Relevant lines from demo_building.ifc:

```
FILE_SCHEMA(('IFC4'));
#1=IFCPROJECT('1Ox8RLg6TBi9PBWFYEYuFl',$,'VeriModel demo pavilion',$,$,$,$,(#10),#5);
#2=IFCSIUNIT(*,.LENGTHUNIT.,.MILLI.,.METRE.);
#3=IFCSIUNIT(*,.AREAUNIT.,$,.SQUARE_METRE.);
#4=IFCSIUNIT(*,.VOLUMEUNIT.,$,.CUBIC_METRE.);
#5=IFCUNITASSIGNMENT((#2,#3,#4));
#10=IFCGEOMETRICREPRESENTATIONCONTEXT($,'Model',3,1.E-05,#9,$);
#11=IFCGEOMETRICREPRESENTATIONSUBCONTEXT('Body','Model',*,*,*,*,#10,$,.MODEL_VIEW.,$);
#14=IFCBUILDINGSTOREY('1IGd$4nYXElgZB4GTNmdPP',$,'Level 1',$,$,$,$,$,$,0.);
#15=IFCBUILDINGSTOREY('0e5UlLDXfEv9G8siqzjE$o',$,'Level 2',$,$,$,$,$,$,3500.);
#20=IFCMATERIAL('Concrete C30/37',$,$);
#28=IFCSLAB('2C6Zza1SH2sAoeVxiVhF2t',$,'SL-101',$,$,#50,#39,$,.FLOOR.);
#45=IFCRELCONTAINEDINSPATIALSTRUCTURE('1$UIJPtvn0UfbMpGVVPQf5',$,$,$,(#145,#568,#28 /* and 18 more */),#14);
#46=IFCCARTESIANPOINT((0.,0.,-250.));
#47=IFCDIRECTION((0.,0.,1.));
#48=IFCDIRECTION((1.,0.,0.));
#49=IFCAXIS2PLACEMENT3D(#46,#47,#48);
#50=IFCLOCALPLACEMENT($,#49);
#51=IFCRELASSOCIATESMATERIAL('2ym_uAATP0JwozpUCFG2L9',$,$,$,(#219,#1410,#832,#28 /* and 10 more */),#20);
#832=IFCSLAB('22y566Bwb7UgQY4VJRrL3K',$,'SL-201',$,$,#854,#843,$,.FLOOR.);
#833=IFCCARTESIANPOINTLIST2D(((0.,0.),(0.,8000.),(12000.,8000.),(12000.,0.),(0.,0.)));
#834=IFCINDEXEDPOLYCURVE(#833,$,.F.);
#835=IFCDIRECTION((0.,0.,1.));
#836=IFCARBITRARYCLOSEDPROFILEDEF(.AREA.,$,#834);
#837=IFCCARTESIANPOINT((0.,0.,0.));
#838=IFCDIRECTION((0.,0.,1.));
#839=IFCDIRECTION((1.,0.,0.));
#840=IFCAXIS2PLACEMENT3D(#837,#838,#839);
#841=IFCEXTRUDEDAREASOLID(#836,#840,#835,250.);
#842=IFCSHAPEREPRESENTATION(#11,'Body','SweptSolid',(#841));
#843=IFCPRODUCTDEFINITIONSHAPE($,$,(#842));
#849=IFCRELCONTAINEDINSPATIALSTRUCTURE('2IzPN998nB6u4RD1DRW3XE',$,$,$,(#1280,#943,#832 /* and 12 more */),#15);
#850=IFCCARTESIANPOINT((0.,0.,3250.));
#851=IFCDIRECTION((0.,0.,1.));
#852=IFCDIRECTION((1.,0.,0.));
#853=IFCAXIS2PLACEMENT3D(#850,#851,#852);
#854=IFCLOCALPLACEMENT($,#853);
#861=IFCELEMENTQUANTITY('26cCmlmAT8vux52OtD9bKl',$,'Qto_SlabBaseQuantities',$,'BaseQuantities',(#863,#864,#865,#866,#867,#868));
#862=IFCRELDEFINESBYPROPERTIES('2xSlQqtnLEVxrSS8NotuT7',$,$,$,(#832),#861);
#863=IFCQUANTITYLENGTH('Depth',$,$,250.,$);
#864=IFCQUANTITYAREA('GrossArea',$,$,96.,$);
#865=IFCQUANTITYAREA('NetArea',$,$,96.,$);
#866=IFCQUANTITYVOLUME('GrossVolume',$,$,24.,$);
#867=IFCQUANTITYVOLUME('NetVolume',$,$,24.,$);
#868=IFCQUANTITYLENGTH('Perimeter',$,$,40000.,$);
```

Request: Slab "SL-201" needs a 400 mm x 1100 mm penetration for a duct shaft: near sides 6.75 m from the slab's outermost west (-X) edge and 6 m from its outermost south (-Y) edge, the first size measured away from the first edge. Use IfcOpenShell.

```python
import numpy as np
import ifcopenshell
import ifcopenshell.api.feature
import ifcopenshell.api.geometry
import ifcopenshell.api.pset
import ifcopenshell.api.root
import ifcopenshell.geom
import ifcopenshell.util.element
import ifcopenshell.util.placement
import ifcopenshell.util.representation
import ifcopenshell.util.shape
import ifcopenshell.util.unit

model = ifcopenshell.open("demo_building.ifc")
unit_scale = ifcopenshell.util.unit.calculate_unit_scale(model)
area_scale = ifcopenshell.util.unit.calculate_unit_scale(model, "AREAUNIT")
volume_scale = ifcopenshell.util.unit.calculate_unit_scale(model, "VOLUMEUNIT")
settings = ifcopenshell.geom.settings()


def volume(element):
    """Net volume in cubic metres, openings subtracted."""
    shape = ifcopenshell.geom.create_shape(settings, element)
    return ifcopenshell.util.shape.get_volume(shape.geometry)


slab = model.by_guid("22y566Bwb7UgQY4VJRrL3K")
before = volume(slab)

# Extent in the slab's own axes, in metres. The edges named are its -X and -Y sides.
slab_shape = ifcopenshell.geom.create_shape(settings, slab)
vertices = ifcopenshell.util.shape.get_vertices(slab_shape.geometry)
x_min, y_min, bottom = vertices.min(axis=0)
top = vertices[:, 2].max()

opening = ifcopenshell.api.root.create_entity(model, ifc_class="IfcOpeningElement", name="Duct shaft opening", predefined_type="OPENING")
context = ifcopenshell.util.representation.get_context(model, "Model", "Body", "MODEL_VIEW")
width, depth = 0.4, 1.1
outline = [(0.0, 0.0), (width, 0.0), (width, depth), (0.0, depth), (0.0, 0.0)]
# Overshoot both faces by 50 mm so the cut is clean.
shape = ifcopenshell.api.geometry.add_slab_representation(
    model, context=context, depth=top - bottom + 0.1, polyline=outline
)
ifcopenshell.api.geometry.assign_representation(model, product=opening, representation=shape)

matrix = ifcopenshell.util.placement.get_local_placement(slab.ObjectPlacement)
matrix[:, 3] = matrix @ np.append(np.array([x_min + 6.75, y_min + 6, bottom - 0.05]) / unit_scale, 1.0)
ifcopenshell.api.geometry.edit_object_placement(model, product=opening, matrix=matrix, is_si=False)
ifcopenshell.api.feature.add_feature(model, feature=opening, element=slab)

after = volume(slab)

# Update the slab's stored quantities.
qto = model.by_id(ifcopenshell.util.element.get_pset(slab, "Qto_SlabBaseQuantities", should_inherit=False)["id"])
ifcopenshell.api.pset.edit_qto(model, qto=qto, properties={
    "NetArea": after / (top - bottom) / area_scale,
    "NetVolume": after / volume_scale,
})

print(f"slab volume {before:.3f} -> {after:.3f} m3")

model.write("demo_building_v2.ifc")
```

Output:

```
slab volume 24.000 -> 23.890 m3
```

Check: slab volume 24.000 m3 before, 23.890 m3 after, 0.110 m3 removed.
